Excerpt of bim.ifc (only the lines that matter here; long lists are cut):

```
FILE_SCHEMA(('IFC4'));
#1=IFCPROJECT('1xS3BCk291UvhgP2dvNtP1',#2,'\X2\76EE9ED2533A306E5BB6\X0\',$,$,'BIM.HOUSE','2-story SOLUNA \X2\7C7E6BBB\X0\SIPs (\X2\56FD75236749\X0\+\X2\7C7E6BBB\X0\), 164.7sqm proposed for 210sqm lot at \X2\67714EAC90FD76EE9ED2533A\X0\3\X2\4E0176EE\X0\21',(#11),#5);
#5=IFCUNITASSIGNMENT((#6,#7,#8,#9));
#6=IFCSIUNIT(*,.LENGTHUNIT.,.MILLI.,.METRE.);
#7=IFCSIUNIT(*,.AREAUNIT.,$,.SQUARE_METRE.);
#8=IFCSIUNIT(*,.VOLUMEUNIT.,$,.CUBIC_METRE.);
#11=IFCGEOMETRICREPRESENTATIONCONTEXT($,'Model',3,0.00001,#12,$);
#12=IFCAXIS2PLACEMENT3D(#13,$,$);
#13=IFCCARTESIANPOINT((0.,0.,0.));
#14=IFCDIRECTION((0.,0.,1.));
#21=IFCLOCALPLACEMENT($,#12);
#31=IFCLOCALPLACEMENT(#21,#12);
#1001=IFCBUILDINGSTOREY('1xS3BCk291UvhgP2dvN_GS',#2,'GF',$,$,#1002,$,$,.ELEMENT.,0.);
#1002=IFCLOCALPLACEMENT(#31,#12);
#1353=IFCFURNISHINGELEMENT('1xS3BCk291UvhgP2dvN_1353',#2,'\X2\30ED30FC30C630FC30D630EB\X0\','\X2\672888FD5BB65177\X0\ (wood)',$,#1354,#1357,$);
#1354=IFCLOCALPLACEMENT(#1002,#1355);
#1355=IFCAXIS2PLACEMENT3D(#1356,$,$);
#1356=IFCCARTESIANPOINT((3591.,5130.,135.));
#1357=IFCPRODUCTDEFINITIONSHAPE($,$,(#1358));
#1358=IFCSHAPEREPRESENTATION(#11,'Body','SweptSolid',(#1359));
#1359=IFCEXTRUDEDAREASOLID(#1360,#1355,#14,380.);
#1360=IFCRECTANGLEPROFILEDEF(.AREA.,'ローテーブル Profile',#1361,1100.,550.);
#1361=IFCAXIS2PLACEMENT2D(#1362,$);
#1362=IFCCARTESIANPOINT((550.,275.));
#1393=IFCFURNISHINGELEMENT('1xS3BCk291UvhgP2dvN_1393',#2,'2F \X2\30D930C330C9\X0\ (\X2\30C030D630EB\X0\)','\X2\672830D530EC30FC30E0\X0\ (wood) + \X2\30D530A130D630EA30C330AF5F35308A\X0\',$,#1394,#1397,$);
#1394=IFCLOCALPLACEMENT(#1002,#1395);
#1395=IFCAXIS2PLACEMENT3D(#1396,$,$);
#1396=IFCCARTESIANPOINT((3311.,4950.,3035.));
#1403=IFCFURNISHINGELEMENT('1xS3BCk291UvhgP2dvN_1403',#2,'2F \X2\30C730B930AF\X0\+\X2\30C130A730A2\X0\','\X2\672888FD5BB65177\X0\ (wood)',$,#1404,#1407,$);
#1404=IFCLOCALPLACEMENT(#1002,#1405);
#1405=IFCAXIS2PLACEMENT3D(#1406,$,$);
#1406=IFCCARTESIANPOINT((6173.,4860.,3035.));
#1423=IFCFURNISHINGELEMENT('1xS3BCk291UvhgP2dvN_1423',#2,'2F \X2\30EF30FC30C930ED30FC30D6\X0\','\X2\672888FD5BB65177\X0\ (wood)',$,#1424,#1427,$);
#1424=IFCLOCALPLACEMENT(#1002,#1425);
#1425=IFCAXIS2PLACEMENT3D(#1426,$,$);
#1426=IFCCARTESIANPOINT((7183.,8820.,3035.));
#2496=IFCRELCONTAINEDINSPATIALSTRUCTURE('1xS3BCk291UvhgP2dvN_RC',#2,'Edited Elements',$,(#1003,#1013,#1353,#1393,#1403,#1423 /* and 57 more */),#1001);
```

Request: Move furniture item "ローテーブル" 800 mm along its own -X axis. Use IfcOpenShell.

```python
import ifcopenshell
import ifcopenshell.api.geometry
import ifcopenshell.util.placement
import ifcopenshell.util.unit

model = ifcopenshell.open("bim.ifc")
unit_scale = ifcopenshell.util.unit.calculate_unit_scale(model)

item = model.by_guid("1xS3BCk291UvhgP2dvN_1353")
matrix = ifcopenshell.util.placement.get_local_placement(item.ObjectPlacement)
matrix[:3, 3] -= matrix[:3, 0] * 0.8 / unit_scale
ifcopenshell.api.geometry.edit_object_placement(model, product=item, matrix=matrix, is_si=False)

print(ifcopenshell.util.placement.get_local_placement(item.ObjectPlacement).round(3) + 0.0)

model.write("bim_updated.ifc")
```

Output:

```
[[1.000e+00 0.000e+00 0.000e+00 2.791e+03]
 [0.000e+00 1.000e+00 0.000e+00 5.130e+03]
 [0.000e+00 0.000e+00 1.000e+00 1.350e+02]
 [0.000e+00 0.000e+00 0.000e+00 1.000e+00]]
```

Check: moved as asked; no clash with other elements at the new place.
